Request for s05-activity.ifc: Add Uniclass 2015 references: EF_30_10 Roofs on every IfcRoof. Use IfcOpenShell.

First a look at what the model holds.

```python
import ifcopenshell

model = ifcopenshell.open("s05-activity.ifc")
print(model.schema)
print("classifications:", [c.Name for c in model.by_type("IfcClassification")])
for ifc_class in ("IfcDoor", "IfcRoof", "IfcStair", "IfcWall", "IfcWindow"):
    print(ifc_class, len(model.by_type(ifc_class)))
```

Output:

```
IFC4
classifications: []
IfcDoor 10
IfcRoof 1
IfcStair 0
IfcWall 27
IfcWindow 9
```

```python
import ifcopenshell
import ifcopenshell.api.classification

model = ifcopenshell.open("s05-activity.ifc")

system = ifcopenshell.api.classification.add_classification(model, classification="Uniclass 2015")

codes = {
    "IfcRoof": ("EF_30_10", "Roofs"),
}
for ifc_class, (code, name) in codes.items():
    products = model.by_type(ifc_class)
    ifcopenshell.api.classification.add_reference(
        model, products=products, classification=system, identification=code, name=name
    )
    print(code, len(products))

model.write("s05-activity_updated.ifc")
```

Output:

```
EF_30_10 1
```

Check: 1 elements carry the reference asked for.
